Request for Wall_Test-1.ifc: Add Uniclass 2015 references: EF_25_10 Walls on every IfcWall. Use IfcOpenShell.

First a look at what the model holds.

```python
import ifcopenshell

model = ifcopenshell.open("Wall_Test-1.ifc")
print(model.schema)
print("classifications:", [c.Name for c in model.by_type("IfcClassification")])
for ifc_class in ("IfcDoor", "IfcRoof", "IfcStair", "IfcWall", "IfcWindow"):
    print(ifc_class, len(model.by_type(ifc_class)))
```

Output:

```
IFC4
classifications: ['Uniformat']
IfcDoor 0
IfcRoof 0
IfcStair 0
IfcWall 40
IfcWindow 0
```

```python
import ifcopenshell
import ifcopenshell.api.classification

model = ifcopenshell.open("Wall_Test-1.ifc")

system = ifcopenshell.api.classification.add_classification(model, classification="Uniclass 2015")

codes = {
    "IfcWall": ("EF_25_10", "Walls"),
}
for ifc_class, (code, name) in codes.items():
    products = model.by_type(ifc_class)
    ifcopenshell.api.classification.add_reference(
        model, products=products, classification=system, identification=code, name=name
    )
    print(code, len(products))

model.write("Wall_Test-1_v2.ifc")
```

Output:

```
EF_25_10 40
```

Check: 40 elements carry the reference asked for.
